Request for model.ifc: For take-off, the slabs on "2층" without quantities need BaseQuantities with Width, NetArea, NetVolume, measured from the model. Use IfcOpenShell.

First a look at what the model holds.

```python
import ifcopenshell
import ifcopenshell.util.element
import ifcopenshell.util.unit

model = ifcopenshell.open("model.ifc")
print(model.schema)
for unit_type in ("LENGTHUNIT", "AREAUNIT", "VOLUMEUNIT"):
    print(unit_type, ifcopenshell.util.unit.calculate_unit_scale(model, unit_type))
storey = next(s for s in model.by_type("IfcBuildingStorey") if s.Name == "2층")
slabs = [e for e in ifcopenshell.util.element.get_decomposition(storey) if e.is_a("IfcSlab")]
for e in sorted(slabs, key=lambda e: e.id()):
    print(e.id(), e.is_a(), e.Name, list(ifcopenshell.util.element.get_psets(e, qtos_only=True)), sep=" | ")
```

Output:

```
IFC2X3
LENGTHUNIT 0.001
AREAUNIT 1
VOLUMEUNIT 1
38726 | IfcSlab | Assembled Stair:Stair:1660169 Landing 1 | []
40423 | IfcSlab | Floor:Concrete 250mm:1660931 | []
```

```python
import ifcopenshell
import ifcopenshell.api.pset
import ifcopenshell.geom
import ifcopenshell.util.element
import ifcopenshell.util.shape
import ifcopenshell.util.unit

model = ifcopenshell.open("model.ifc")
unit_scale = ifcopenshell.util.unit.calculate_unit_scale(model)
area_scale = ifcopenshell.util.unit.calculate_unit_scale(model, "AREAUNIT")
volume_scale = ifcopenshell.util.unit.calculate_unit_scale(model, "VOLUMEUNIT")
settings = ifcopenshell.geom.settings()

storey = next(s for s in model.by_type("IfcBuildingStorey") if s.Name == "2층")
slabs = [e for e in ifcopenshell.util.element.get_decomposition(storey) if e.is_a("IfcSlab")]

for e in sorted(slabs, key=lambda e: e.id()):
    if ifcopenshell.util.element.get_psets(e, qtos_only=True, should_inherit=False):
        continue
    # Geometry comes back in metres, in the element's own axes.
    shape = ifcopenshell.geom.create_shape(settings, e)
    values = {
        "Width": ifcopenshell.util.shape.get_z(shape.geometry) / unit_scale,
        "NetArea": ifcopenshell.util.shape.get_footprint_area(shape.geometry) / area_scale,
        "NetVolume": ifcopenshell.util.shape.get_volume(shape.geometry) / volume_scale,
    }
    qto = ifcopenshell.api.pset.add_qto(model, product=e, name="BaseQuantities")
    ifcopenshell.api.pset.edit_qto(model, qto=qto, properties=values)
    print(e.id(), {k: round(v, 3) for k, v in values.items()})

model.write("model-out.ifc")
```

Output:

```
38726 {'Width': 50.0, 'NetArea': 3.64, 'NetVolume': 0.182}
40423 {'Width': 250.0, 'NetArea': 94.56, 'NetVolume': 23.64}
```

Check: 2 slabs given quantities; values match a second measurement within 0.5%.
